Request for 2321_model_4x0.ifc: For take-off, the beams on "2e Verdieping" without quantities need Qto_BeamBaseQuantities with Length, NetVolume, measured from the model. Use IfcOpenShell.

First a look at what the model holds.

```python
import ifcopenshell
import ifcopenshell.util.element
import ifcopenshell.util.unit

model = ifcopenshell.open("2321_model_4x0.ifc")
print(model.schema)
for unit_type in ("LENGTHUNIT", "AREAUNIT", "VOLUMEUNIT"):
    print(unit_type, ifcopenshell.util.unit.calculate_unit_scale(model, unit_type))
storey = next(s for s in model.by_type("IfcBuildingStorey") if s.Name == "2e Verdieping")
beams = [e for e in ifcopenshell.util.element.get_decomposition(storey) if e.is_a("IfcBeam")]
for e in sorted(beams, key=lambda e: e.id()):
    print(e.id(), e.is_a(), e.Name, list(ifcopenshell.util.element.get_psets(e, qtos_only=True)), sep=" | ")
```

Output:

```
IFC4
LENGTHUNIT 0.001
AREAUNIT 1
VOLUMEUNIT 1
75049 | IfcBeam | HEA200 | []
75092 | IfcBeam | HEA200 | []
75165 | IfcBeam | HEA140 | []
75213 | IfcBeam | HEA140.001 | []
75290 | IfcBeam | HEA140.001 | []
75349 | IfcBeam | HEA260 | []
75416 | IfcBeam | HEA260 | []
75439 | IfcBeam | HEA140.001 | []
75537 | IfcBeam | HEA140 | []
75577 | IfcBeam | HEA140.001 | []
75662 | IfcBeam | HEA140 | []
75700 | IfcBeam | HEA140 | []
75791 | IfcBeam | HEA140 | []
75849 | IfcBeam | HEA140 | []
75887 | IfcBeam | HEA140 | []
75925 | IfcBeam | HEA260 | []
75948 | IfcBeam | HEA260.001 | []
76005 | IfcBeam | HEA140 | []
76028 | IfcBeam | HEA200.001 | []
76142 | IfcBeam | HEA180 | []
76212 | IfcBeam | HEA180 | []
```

```python
import ifcopenshell
import ifcopenshell.api.pset
import ifcopenshell.geom
import ifcopenshell.util.element
import ifcopenshell.util.shape
import ifcopenshell.util.unit

model = ifcopenshell.open("2321_model_4x0.ifc")
unit_scale = ifcopenshell.util.unit.calculate_unit_scale(model)
volume_scale = ifcopenshell.util.unit.calculate_unit_scale(model, "VOLUMEUNIT")
settings = ifcopenshell.geom.settings()

storey = next(s for s in model.by_type("IfcBuildingStorey") if s.Name == "2e Verdieping")
beams = [e for e in ifcopenshell.util.element.get_decomposition(storey) if e.is_a("IfcBeam")]

for e in sorted(beams, key=lambda e: e.id()):
    if ifcopenshell.util.element.get_psets(e, qtos_only=True, should_inherit=False):
        continue
    # Geometry comes back in metres, in the element's own axes.
    shape = ifcopenshell.geom.create_shape(settings, e)
    values = {
        "Length": ifcopenshell.util.shape.get_max_xyz(shape.geometry) / unit_scale,
        "NetVolume": ifcopenshell.util.shape.get_volume(shape.geometry) / volume_scale,
    }
    qto = ifcopenshell.api.pset.add_qto(model, product=e, name="Qto_BeamBaseQuantities")
    ifcopenshell.api.pset.edit_qto(model, qto=qto, properties=values)
    print(e.id(), {k: round(v, 3) for k, v in values.items()})

model.write("2321_model_4x0_rev.ifc")
```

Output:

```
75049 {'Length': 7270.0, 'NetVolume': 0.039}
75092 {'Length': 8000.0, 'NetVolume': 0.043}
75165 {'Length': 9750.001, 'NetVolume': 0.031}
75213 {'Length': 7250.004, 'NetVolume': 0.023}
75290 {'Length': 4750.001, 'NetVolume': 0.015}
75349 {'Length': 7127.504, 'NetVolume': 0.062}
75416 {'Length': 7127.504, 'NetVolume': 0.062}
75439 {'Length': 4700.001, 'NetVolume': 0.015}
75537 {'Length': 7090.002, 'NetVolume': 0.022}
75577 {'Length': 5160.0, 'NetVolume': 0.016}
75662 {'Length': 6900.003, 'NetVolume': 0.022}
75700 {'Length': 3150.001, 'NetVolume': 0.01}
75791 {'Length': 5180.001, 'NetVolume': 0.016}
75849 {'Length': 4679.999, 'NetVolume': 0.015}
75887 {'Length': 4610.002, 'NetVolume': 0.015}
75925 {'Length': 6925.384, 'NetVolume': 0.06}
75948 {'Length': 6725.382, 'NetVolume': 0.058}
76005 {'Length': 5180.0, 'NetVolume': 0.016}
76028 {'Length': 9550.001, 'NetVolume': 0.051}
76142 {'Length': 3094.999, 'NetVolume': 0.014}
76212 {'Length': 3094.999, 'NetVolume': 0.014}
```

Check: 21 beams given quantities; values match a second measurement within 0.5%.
